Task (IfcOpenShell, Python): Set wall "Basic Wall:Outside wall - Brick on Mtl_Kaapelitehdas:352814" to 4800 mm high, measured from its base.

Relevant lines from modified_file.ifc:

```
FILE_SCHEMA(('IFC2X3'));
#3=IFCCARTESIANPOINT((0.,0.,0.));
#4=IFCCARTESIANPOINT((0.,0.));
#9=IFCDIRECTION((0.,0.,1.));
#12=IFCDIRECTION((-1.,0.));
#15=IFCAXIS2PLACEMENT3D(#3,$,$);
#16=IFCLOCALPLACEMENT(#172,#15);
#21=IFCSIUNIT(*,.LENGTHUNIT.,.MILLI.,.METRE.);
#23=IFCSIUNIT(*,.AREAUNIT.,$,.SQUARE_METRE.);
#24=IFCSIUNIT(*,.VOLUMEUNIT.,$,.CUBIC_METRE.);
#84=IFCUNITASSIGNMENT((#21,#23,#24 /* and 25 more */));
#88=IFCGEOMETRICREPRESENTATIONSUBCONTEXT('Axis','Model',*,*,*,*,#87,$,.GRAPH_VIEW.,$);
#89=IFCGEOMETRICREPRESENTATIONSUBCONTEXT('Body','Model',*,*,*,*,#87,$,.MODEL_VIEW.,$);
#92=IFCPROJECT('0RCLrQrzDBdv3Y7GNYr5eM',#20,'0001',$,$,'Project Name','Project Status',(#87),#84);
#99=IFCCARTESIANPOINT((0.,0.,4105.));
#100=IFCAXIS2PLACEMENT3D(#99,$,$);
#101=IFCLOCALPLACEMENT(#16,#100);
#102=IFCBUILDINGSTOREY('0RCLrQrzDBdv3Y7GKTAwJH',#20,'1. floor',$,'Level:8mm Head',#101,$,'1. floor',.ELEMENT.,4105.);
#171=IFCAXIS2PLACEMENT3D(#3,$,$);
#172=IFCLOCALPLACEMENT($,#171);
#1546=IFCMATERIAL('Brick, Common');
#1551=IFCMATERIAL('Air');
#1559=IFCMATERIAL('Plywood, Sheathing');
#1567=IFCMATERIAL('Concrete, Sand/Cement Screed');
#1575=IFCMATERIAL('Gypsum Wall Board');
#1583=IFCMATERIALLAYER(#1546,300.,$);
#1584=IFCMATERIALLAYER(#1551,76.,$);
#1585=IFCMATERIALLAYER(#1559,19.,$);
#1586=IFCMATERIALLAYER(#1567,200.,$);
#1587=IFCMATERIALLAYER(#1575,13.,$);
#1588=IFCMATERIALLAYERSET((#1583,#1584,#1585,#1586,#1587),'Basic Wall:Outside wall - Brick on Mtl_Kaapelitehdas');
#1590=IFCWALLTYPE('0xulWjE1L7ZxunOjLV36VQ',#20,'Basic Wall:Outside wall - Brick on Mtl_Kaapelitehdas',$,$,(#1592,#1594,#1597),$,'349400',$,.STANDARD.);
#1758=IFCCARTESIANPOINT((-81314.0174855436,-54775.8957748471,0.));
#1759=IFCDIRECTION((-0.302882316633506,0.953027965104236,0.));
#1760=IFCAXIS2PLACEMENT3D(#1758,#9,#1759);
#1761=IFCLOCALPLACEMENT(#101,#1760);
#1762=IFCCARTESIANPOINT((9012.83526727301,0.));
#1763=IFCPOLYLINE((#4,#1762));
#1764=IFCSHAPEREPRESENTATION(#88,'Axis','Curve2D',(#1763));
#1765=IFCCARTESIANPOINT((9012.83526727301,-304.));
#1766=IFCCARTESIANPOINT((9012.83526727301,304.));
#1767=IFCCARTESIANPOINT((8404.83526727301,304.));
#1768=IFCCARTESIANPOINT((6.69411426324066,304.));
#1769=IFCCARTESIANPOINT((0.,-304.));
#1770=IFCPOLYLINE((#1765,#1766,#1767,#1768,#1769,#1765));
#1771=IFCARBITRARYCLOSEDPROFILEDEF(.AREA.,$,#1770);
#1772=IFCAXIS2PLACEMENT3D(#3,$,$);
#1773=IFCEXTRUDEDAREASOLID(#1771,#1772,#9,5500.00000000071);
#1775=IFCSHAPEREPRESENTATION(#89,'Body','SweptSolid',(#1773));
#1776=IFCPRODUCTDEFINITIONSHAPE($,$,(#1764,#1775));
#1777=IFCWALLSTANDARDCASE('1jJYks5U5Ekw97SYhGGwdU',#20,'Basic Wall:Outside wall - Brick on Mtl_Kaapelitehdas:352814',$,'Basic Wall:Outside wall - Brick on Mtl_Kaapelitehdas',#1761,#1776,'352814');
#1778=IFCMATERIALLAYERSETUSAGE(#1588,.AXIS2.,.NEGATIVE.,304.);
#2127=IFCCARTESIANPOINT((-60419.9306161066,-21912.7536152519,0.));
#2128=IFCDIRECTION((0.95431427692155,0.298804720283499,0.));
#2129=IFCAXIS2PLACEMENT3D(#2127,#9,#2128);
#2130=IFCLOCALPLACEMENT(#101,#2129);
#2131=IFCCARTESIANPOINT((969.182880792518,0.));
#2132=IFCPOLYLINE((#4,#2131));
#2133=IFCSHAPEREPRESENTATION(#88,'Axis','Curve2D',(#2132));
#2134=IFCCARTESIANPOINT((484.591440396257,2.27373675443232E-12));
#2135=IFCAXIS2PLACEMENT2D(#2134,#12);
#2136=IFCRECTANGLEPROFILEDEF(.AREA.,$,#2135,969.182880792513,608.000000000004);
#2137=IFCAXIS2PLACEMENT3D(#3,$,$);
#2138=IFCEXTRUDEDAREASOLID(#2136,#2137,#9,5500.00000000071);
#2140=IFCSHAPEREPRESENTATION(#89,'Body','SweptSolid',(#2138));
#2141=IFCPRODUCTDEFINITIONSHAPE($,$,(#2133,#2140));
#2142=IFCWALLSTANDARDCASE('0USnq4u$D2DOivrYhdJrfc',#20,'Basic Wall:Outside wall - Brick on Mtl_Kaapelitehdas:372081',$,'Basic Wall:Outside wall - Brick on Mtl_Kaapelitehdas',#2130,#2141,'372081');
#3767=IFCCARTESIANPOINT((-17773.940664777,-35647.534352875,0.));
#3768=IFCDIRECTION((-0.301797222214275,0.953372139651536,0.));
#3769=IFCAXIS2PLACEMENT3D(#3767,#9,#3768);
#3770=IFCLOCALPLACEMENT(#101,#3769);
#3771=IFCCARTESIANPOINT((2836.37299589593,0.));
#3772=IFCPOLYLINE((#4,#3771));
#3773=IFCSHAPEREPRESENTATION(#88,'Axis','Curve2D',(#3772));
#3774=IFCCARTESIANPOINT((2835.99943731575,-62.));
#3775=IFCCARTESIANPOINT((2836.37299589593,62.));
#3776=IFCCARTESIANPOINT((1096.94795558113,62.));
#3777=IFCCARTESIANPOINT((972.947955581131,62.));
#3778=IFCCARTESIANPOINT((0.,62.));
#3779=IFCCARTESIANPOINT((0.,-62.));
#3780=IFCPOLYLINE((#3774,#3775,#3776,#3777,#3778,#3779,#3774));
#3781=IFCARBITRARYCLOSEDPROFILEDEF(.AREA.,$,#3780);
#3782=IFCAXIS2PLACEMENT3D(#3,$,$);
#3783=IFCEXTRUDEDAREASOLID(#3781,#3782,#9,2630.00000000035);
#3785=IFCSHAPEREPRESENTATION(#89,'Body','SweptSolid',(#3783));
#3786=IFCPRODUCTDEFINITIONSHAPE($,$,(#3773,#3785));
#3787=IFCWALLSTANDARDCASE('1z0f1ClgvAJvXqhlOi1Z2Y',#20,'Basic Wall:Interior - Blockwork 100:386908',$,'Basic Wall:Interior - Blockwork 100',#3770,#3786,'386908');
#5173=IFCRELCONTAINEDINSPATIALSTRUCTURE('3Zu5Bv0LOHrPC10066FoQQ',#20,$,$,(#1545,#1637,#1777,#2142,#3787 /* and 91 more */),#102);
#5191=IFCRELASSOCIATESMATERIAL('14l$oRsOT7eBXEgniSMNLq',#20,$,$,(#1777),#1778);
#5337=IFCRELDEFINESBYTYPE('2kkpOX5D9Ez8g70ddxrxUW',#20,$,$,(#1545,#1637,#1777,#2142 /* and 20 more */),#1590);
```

```python
import ifcopenshell
import ifcopenshell.geom
import ifcopenshell.util.representation
import ifcopenshell.util.shape

model = ifcopenshell.open("modified_file.ifc")
settings = ifcopenshell.geom.settings()


def volume(element):
    """Net volume in cubic metres, openings subtracted."""
    shape = ifcopenshell.geom.create_shape(settings, element)
    return ifcopenshell.util.shape.get_volume(shape.geometry)


wall = model.by_id(1777)
before = volume(wall)

body = ifcopenshell.util.representation.get_representation(wall, "Model", "Body")
solid = body.Items[0]
old_height = solid.Depth
solid.Depth = 4800.0
after = volume(wall)

print(f"height {old_height:g} -> {solid.Depth:g}, volume {before:.3f} -> {after:.3f} m3")

model.write("modified_file_rev.ifc")
```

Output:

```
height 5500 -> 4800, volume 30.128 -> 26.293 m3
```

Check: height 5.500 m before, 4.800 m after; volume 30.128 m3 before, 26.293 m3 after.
